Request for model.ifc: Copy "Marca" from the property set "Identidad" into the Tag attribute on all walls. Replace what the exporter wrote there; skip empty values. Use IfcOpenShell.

First a look at what the model holds.

```python
import ifcopenshell
import ifcopenshell.util.element

model = ifcopenshell.open("model.ifc")
print(model.schema)
walls = model.by_type("IfcWall")
print(len(walls), "walls")
for e in walls[:8]:
    source = ifcopenshell.util.element.get_pset(e, "Identidad", "Marca")
    target = e.Tag
    print(e.id(), repr(source), repr(target), sep=" | ")
```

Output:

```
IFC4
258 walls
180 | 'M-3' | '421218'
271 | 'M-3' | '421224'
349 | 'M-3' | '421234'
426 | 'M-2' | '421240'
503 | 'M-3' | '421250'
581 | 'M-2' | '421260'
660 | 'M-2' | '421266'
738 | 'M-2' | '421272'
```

```python
import ifcopenshell
import ifcopenshell.util.element

model = ifcopenshell.open("model.ifc")

count = 0
for e in model.by_type("IfcWall"):
    value = ifcopenshell.util.element.get_pset(e, "Identidad", "Marca")
    current = e.Tag
    if not value or not value.strip() or current == value:
        continue
    e.Tag = value
    count += 1

print(count, "walls updated")

model.write("model_v2.ifc")
```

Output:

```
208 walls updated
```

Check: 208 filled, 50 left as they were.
